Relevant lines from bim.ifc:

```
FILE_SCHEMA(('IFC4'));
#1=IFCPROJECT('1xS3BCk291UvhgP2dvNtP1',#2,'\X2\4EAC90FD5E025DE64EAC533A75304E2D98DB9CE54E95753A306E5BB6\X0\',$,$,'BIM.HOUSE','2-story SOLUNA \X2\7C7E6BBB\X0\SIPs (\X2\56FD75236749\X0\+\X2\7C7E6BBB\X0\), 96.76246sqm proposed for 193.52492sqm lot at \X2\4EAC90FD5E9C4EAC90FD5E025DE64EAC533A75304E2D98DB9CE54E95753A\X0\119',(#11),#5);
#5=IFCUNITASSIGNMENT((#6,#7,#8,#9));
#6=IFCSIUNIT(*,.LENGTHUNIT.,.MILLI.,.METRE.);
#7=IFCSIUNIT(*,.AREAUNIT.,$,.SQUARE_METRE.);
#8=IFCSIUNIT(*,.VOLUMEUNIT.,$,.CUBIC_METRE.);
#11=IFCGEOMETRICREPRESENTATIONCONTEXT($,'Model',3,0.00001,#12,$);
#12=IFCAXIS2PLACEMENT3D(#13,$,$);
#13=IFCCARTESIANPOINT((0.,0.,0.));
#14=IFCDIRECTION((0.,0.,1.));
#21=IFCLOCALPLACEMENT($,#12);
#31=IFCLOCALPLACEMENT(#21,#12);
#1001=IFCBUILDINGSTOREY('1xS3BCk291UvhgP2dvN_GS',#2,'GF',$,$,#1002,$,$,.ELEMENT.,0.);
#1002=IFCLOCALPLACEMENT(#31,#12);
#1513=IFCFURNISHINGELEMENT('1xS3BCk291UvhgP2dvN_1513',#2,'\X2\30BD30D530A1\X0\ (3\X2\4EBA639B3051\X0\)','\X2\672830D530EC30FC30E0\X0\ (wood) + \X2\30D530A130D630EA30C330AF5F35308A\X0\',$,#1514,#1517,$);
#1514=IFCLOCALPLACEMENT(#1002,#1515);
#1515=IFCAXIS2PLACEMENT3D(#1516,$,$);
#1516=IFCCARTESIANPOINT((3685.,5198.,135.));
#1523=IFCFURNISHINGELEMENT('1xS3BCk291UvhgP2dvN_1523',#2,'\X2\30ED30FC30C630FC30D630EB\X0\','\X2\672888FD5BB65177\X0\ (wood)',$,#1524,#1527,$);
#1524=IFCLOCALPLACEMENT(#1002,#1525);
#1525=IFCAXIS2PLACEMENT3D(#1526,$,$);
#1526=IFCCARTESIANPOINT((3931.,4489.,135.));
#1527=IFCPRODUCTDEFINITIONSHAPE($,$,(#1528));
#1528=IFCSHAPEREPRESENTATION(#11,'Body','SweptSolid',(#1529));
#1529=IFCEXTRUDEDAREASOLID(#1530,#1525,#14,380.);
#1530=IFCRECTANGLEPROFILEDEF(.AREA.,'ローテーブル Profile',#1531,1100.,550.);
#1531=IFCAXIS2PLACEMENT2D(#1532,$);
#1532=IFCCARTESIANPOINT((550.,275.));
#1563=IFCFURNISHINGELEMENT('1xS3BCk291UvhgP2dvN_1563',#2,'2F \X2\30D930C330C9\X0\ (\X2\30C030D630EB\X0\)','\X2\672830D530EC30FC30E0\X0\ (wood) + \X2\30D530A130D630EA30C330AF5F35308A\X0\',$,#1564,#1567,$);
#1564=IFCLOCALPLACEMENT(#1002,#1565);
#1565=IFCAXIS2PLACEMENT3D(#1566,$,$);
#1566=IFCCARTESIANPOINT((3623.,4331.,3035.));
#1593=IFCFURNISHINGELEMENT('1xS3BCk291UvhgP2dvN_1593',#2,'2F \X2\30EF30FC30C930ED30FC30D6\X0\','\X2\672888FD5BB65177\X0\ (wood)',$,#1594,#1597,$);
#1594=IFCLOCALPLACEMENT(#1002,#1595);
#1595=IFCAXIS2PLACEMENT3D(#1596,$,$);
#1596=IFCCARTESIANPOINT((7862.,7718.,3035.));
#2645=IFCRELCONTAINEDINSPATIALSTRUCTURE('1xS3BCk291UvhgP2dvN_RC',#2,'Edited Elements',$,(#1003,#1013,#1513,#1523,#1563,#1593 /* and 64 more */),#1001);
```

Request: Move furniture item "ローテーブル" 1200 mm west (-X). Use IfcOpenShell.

```python
import ifcopenshell
import ifcopenshell.api.geometry
import ifcopenshell.util.placement
import ifcopenshell.util.unit

model = ifcopenshell.open("bim.ifc")
unit_scale = ifcopenshell.util.unit.calculate_unit_scale(model)

item = model.by_guid("1xS3BCk291UvhgP2dvN_1523")
matrix = ifcopenshell.util.placement.get_local_placement(item.ObjectPlacement)
matrix[0, 3] -= 1.2 / unit_scale
ifcopenshell.api.geometry.edit_object_placement(model, product=item, matrix=matrix, is_si=False)

print(ifcopenshell.util.placement.get_local_placement(item.ObjectPlacement).round(3) + 0.0)

model.write("bim_rev.ifc")
```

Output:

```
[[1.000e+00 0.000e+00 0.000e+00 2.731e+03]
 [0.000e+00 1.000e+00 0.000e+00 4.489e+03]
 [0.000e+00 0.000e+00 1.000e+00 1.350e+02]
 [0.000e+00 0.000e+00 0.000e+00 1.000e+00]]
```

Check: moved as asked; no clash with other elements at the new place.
